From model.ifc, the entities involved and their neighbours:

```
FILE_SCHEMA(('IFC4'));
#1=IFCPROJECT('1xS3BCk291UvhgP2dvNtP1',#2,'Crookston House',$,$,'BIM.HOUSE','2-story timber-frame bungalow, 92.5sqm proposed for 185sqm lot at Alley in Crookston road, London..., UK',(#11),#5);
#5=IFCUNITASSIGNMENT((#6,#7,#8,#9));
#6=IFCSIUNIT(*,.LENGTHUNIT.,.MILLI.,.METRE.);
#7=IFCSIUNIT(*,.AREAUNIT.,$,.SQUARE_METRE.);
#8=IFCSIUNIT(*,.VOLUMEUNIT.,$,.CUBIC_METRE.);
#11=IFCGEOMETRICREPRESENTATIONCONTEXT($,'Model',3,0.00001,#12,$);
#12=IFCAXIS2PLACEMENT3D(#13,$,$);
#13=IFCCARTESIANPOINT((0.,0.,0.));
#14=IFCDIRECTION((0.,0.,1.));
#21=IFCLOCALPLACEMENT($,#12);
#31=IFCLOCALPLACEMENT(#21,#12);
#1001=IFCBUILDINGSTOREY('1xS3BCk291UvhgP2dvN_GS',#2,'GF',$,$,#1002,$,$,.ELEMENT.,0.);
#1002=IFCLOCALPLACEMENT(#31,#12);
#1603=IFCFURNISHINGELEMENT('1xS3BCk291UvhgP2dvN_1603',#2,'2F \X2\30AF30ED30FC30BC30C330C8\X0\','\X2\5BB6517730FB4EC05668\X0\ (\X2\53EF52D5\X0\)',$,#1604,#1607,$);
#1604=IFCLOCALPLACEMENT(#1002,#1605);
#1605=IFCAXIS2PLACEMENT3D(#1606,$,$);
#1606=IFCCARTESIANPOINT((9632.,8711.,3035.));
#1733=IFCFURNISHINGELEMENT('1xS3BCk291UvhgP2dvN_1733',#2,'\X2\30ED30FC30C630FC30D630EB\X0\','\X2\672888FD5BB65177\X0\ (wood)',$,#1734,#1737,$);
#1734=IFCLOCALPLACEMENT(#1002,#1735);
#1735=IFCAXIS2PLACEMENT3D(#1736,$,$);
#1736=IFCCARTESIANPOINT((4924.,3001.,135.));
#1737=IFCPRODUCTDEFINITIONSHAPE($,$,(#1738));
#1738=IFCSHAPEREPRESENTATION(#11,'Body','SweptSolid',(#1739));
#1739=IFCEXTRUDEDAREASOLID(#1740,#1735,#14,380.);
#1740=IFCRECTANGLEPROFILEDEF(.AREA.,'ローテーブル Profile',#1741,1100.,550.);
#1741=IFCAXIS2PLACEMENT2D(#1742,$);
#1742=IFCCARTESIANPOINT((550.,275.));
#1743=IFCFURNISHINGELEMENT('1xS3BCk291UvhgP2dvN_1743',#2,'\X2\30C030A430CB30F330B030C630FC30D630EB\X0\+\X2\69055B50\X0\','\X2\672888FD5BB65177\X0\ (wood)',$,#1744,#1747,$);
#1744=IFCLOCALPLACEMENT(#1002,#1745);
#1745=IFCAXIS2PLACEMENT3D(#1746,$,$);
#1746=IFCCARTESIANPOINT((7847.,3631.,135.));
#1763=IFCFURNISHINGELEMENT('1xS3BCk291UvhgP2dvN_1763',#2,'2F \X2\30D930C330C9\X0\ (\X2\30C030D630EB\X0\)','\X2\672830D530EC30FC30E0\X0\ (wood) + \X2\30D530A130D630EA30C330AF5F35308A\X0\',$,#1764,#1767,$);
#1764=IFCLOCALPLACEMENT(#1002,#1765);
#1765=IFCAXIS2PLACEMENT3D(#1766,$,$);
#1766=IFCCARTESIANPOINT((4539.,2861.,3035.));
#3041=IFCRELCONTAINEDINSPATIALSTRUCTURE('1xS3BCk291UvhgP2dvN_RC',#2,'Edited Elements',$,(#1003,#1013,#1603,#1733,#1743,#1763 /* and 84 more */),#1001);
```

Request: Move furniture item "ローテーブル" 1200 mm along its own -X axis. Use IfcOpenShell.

```python
import ifcopenshell
import ifcopenshell.api.geometry
import ifcopenshell.util.placement

model = ifcopenshell.open("model.ifc")

item = model.by_guid("1xS3BCk291UvhgP2dvN_1733")
matrix = ifcopenshell.util.placement.get_local_placement(item.ObjectPlacement)
matrix[:3, 3] -= matrix[:3, 0] * 1200.0
ifcopenshell.api.geometry.edit_object_placement(model, product=item, matrix=matrix, is_si=False)

print(ifcopenshell.util.placement.get_local_placement(item.ObjectPlacement).round(3) + 0.0)

model.write("model_edited.ifc")
```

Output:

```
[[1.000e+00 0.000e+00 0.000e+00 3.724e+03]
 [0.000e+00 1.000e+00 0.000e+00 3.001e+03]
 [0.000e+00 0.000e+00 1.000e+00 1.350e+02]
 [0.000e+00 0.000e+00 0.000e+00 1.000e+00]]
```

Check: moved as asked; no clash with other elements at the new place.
